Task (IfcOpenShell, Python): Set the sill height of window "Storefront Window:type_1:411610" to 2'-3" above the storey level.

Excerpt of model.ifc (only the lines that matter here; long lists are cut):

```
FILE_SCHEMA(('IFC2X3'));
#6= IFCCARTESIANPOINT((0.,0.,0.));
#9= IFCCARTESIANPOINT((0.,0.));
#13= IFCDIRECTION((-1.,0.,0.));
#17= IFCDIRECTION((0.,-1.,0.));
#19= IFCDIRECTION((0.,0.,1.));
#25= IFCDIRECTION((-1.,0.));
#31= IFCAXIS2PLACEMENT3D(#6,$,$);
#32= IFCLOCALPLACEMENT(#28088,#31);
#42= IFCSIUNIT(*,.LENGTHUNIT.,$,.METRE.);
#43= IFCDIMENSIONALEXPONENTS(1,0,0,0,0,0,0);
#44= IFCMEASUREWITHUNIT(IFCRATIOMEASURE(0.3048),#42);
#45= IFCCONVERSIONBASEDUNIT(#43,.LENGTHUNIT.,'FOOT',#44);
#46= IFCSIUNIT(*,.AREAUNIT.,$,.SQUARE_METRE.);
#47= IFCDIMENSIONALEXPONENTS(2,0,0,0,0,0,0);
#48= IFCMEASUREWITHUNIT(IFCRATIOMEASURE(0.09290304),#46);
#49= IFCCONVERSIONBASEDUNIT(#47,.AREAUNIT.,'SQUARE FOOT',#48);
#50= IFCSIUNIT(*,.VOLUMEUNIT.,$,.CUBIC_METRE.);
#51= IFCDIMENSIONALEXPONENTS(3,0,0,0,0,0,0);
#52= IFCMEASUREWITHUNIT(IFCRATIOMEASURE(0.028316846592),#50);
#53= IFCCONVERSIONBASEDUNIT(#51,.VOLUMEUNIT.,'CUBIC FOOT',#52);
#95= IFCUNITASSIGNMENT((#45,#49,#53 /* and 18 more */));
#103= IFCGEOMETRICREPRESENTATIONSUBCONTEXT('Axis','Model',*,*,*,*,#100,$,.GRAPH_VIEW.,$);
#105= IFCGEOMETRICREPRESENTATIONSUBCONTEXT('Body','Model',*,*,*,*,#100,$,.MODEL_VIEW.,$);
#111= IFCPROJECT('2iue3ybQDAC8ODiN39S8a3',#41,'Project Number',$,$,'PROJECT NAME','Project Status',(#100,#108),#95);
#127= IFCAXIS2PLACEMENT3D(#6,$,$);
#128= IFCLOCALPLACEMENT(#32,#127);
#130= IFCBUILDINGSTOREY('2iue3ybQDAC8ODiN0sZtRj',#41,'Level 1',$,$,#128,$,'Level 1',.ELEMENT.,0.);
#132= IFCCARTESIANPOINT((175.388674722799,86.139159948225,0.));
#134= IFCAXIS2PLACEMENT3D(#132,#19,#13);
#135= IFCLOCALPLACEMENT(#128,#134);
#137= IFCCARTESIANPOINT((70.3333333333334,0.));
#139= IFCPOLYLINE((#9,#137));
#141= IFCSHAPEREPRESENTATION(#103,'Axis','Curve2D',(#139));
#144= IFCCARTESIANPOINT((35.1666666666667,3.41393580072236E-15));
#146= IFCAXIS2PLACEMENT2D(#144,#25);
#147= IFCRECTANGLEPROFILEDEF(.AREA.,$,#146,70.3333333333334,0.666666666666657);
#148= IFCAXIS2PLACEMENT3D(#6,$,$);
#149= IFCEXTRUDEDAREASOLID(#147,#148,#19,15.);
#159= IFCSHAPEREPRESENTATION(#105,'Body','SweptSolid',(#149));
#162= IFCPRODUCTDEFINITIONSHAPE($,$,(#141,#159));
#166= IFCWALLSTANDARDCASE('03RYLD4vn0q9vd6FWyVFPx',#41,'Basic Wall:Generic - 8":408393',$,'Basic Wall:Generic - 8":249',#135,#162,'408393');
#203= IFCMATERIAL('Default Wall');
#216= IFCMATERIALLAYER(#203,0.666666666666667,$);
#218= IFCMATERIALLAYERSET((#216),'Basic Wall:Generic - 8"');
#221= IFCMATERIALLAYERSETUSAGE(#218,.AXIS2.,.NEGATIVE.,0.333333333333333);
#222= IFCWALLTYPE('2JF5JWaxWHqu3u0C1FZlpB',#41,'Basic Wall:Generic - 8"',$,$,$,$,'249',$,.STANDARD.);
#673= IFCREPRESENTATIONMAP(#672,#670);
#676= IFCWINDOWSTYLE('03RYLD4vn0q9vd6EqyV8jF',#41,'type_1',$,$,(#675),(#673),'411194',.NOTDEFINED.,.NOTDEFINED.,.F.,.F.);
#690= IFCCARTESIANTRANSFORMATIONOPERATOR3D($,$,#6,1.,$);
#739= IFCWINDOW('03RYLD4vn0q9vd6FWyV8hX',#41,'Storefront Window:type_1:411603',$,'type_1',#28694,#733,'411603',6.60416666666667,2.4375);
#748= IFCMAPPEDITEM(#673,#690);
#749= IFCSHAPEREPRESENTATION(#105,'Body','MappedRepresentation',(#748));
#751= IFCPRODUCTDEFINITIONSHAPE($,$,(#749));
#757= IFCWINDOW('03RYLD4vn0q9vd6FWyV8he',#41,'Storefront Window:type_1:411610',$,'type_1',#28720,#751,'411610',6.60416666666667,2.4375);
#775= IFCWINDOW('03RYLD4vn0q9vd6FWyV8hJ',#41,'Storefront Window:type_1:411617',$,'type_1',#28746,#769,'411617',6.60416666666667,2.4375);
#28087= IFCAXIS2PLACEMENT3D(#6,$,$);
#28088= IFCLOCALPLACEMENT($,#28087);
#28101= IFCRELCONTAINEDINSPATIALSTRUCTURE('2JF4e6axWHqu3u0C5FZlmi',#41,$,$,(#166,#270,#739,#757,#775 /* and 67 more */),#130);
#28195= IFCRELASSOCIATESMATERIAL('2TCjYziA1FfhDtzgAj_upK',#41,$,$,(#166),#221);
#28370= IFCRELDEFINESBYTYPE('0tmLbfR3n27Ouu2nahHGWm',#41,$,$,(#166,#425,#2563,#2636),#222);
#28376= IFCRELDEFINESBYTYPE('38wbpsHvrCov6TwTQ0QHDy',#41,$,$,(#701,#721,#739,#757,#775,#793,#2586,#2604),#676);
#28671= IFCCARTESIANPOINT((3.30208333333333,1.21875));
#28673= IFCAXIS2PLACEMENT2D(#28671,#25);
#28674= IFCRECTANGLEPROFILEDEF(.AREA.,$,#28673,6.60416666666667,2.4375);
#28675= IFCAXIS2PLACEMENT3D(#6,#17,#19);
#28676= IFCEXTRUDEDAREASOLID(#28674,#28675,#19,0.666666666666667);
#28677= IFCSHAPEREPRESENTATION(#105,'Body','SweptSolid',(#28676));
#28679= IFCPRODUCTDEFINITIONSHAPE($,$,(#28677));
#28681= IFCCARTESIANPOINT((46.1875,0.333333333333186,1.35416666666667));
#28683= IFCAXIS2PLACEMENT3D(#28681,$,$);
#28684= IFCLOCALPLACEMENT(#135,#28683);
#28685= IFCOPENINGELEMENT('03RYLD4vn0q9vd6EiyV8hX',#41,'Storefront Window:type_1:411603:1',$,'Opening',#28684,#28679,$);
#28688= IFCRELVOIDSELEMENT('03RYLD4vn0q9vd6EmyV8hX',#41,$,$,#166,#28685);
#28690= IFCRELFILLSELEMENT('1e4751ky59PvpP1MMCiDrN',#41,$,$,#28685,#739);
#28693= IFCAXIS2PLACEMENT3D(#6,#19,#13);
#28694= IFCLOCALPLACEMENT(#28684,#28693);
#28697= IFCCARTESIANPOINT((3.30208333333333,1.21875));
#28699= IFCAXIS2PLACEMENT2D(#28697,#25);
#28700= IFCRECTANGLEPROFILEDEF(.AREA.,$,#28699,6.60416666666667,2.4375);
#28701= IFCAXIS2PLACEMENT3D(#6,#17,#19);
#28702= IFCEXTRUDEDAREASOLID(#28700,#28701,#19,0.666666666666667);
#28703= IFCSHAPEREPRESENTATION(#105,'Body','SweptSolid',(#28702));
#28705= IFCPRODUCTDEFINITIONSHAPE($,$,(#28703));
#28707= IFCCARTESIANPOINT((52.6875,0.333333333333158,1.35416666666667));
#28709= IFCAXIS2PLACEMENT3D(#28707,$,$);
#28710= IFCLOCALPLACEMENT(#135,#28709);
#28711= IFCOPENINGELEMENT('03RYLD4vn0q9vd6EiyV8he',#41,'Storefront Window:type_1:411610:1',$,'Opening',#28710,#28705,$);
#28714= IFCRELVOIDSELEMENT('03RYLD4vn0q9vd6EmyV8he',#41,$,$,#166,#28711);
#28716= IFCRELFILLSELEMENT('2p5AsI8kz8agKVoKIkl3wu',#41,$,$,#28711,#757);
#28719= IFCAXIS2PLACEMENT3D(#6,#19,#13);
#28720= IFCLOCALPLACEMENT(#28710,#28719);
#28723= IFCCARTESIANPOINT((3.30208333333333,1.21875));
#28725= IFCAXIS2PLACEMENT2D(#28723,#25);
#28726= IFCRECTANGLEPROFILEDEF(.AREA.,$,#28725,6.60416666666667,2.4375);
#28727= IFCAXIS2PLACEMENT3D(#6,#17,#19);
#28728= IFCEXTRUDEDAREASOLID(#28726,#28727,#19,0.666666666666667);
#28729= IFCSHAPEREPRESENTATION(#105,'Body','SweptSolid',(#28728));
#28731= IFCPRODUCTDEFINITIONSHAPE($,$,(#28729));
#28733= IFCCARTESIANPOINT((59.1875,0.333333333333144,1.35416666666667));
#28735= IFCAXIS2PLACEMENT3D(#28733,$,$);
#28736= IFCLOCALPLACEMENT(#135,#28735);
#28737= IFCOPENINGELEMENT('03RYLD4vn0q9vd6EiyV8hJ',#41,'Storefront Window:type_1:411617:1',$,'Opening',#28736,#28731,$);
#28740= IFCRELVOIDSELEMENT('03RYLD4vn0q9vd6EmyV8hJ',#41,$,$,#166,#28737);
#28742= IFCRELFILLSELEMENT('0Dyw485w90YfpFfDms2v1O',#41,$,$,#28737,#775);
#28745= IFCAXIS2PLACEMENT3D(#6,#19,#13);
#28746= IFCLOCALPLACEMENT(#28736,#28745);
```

```python
import numpy as np
import ifcopenshell
import ifcopenshell.api.geometry
import ifcopenshell.geom
import ifcopenshell.util.element
import ifcopenshell.util.placement
import ifcopenshell.util.shape
import ifcopenshell.util.unit

model = ifcopenshell.open("model.ifc")
unit_scale = ifcopenshell.util.unit.calculate_unit_scale(model)

window = model.by_guid("03RYLD4vn0q9vd6FWyV8he")
opening = window.FillsVoids[0].RelatingOpeningElement
storey = ifcopenshell.util.element.get_container(window, ifc_class="IfcBuildingStorey")
level = ifcopenshell.util.placement.get_local_placement(storey.ObjectPlacement)[2, 3]

# The opening's origin need not be at the sill, so measure its lowest point.
shape = ifcopenshell.geom.create_shape(ifcopenshell.geom.settings(), opening)
bottom = ifcopenshell.util.shape.get_shape_bottom_elevation(shape, shape.geometry) / unit_scale
dz = level + 27 * 0.0254 / unit_scale - bottom

shift = np.array([0.0, 0.0, dz])
# The window is placed relative to its opening, so it follows when the opening moves.
matrix = ifcopenshell.util.placement.get_local_placement(opening.ObjectPlacement)
matrix[:3, 3] += shift
ifcopenshell.api.geometry.edit_object_placement(
    model, product=opening, matrix=matrix, is_si=False, should_transform_children=True
)

print(f"moved by {dz * unit_scale:+.3f} m")

model.write("model_edited.ifc")
```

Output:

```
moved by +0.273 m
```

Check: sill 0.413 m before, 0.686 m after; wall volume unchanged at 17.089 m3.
